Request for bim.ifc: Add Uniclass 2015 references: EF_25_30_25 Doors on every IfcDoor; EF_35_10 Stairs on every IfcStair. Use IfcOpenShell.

First a look at what the model holds.

```python
import ifcopenshell

model = ifcopenshell.open("bim.ifc")
print(model.schema)
print("classifications:", [c.Name for c in model.by_type("IfcClassification")])
for ifc_class in ("IfcDoor", "IfcRoof", "IfcStair", "IfcWall", "IfcWindow"):
    print(ifc_class, len(model.by_type(ifc_class)))
```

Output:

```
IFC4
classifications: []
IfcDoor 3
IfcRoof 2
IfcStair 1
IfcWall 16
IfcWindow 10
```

```python
import ifcopenshell
import ifcopenshell.api.classification

model = ifcopenshell.open("bim.ifc")

system = ifcopenshell.api.classification.add_classification(model, classification="Uniclass 2015")

codes = {
    "IfcDoor": ("EF_25_30_25", "Doors"),
    "IfcStair": ("EF_35_10", "Stairs"),
}
for ifc_class, (code, name) in codes.items():
    products = model.by_type(ifc_class)
    ifcopenshell.api.classification.add_reference(
        model, products=products, classification=system, identification=code, name=name
    )
    print(code, len(products))

model.write("bim_rev.ifc")
```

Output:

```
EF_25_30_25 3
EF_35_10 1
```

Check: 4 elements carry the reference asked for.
